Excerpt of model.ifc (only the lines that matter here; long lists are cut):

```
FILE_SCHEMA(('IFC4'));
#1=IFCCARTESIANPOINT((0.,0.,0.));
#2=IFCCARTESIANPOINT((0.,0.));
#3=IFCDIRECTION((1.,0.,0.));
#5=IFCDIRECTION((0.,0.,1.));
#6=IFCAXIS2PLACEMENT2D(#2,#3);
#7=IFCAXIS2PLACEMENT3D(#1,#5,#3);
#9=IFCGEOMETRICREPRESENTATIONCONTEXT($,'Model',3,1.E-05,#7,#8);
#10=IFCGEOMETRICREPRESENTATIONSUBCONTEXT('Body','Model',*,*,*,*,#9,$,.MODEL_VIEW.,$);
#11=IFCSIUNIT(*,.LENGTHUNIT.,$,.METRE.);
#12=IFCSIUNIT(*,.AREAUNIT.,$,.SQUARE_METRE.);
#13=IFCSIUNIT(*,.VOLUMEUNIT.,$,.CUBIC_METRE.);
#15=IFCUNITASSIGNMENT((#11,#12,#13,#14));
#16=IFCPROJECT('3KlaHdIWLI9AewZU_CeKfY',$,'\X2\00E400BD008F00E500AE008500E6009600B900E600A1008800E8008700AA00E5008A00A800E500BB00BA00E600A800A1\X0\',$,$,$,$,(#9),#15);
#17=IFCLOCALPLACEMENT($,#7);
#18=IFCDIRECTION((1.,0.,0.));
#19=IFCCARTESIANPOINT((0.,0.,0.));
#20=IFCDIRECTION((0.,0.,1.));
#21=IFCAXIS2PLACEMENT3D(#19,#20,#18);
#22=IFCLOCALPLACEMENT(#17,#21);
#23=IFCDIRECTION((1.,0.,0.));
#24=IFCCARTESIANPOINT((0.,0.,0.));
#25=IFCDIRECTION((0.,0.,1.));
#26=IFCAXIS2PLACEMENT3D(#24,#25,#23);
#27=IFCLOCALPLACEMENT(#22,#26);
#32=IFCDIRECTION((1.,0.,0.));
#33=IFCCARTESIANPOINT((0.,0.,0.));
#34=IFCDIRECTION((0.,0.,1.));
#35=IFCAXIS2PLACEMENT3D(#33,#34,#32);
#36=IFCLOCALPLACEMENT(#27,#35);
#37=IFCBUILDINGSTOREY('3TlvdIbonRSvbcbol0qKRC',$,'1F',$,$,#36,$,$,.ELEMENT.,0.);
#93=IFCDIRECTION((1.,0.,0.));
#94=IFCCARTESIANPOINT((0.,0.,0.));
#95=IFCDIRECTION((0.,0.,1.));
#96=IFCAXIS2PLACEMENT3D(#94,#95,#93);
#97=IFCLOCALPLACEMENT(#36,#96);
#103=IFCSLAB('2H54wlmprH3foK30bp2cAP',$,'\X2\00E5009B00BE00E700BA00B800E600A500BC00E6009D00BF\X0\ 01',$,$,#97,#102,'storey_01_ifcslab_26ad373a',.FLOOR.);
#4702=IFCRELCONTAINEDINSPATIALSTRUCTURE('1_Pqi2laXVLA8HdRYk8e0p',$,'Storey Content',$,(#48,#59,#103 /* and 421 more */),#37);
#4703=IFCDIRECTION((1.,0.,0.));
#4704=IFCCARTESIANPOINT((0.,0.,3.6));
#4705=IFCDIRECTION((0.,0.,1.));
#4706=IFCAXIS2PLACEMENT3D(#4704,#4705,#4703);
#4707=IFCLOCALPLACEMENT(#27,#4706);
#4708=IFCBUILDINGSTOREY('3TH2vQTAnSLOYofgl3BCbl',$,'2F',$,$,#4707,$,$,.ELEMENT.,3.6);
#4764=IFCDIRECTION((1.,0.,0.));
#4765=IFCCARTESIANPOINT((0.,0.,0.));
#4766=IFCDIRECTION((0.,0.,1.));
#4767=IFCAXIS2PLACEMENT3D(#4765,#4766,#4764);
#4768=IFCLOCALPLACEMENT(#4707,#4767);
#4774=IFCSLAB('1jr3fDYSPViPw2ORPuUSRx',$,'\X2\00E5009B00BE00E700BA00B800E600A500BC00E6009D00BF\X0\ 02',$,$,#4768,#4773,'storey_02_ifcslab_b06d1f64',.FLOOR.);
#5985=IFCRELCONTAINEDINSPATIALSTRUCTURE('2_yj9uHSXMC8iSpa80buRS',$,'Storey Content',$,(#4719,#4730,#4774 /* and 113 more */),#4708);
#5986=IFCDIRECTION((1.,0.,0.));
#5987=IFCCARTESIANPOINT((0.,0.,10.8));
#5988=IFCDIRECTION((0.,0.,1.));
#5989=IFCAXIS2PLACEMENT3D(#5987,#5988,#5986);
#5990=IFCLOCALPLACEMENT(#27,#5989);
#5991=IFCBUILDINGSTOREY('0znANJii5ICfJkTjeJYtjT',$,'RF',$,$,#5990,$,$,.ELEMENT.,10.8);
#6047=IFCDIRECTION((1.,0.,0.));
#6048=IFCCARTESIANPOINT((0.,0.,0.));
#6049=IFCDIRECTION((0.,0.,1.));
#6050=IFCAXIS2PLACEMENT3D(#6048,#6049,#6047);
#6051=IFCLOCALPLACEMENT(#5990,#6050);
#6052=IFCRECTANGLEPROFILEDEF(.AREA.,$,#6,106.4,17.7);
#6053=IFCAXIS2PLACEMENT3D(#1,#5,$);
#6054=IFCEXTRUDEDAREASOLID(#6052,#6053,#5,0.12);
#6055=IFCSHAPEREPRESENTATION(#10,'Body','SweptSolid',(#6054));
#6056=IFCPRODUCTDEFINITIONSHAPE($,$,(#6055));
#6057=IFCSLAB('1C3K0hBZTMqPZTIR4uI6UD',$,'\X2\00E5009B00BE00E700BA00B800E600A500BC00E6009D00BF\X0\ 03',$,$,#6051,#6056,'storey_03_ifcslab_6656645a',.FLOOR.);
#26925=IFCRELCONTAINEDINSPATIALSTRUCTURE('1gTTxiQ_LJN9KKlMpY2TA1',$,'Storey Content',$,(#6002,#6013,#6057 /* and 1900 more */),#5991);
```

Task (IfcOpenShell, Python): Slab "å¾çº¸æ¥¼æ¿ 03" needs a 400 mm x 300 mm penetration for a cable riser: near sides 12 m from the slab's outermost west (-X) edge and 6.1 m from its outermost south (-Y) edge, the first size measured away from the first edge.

```python
import numpy as np
import ifcopenshell
import ifcopenshell.api.feature
import ifcopenshell.api.geometry
import ifcopenshell.api.root
import ifcopenshell.geom
import ifcopenshell.util.placement
import ifcopenshell.util.representation
import ifcopenshell.util.shape
import ifcopenshell.util.unit

model = ifcopenshell.open("model.ifc")
unit_scale = ifcopenshell.util.unit.calculate_unit_scale(model)
settings = ifcopenshell.geom.settings()


def volume(element):
    """Net volume in cubic metres, openings subtracted."""
    shape = ifcopenshell.geom.create_shape(settings, element)
    return ifcopenshell.util.shape.get_volume(shape.geometry)


slab = model.by_guid("1C3K0hBZTMqPZTIR4uI6UD")
before = volume(slab)

# Extent in the slab's own axes, in metres. The edges named are its -X and -Y sides.
slab_shape = ifcopenshell.geom.create_shape(settings, slab)
vertices = ifcopenshell.util.shape.get_vertices(slab_shape.geometry)
x_min, y_min, bottom = vertices.min(axis=0)
top = vertices[:, 2].max()

opening = ifcopenshell.api.root.create_entity(model, ifc_class="IfcOpeningElement", name="Cable riser opening", predefined_type="OPENING")
context = ifcopenshell.util.representation.get_context(model, "Model", "Body", "MODEL_VIEW")
width, depth = 0.4, 0.3
outline = [(0.0, 0.0), (width, 0.0), (width, depth), (0.0, depth), (0.0, 0.0)]
# Overshoot both faces by 50 mm so the cut is clean.
shape = ifcopenshell.api.geometry.add_slab_representation(
    model, context=context, depth=top - bottom + 0.1, polyline=outline
)
ifcopenshell.api.geometry.assign_representation(model, product=opening, representation=shape)

matrix = ifcopenshell.util.placement.get_local_placement(slab.ObjectPlacement)
matrix[:, 3] = matrix @ np.append(np.array([x_min + 12, y_min + 6.1, bottom - 0.05]) / unit_scale, 1.0)
ifcopenshell.api.geometry.edit_object_placement(model, product=opening, matrix=matrix, is_si=False)
ifcopenshell.api.feature.add_feature(model, feature=opening, element=slab)

after = volume(slab)

print(f"slab volume {before:.3f} -> {after:.3f} m3")

model.write("model-out.ifc")
```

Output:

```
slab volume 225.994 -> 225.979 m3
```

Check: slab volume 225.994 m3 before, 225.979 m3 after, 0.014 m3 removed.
